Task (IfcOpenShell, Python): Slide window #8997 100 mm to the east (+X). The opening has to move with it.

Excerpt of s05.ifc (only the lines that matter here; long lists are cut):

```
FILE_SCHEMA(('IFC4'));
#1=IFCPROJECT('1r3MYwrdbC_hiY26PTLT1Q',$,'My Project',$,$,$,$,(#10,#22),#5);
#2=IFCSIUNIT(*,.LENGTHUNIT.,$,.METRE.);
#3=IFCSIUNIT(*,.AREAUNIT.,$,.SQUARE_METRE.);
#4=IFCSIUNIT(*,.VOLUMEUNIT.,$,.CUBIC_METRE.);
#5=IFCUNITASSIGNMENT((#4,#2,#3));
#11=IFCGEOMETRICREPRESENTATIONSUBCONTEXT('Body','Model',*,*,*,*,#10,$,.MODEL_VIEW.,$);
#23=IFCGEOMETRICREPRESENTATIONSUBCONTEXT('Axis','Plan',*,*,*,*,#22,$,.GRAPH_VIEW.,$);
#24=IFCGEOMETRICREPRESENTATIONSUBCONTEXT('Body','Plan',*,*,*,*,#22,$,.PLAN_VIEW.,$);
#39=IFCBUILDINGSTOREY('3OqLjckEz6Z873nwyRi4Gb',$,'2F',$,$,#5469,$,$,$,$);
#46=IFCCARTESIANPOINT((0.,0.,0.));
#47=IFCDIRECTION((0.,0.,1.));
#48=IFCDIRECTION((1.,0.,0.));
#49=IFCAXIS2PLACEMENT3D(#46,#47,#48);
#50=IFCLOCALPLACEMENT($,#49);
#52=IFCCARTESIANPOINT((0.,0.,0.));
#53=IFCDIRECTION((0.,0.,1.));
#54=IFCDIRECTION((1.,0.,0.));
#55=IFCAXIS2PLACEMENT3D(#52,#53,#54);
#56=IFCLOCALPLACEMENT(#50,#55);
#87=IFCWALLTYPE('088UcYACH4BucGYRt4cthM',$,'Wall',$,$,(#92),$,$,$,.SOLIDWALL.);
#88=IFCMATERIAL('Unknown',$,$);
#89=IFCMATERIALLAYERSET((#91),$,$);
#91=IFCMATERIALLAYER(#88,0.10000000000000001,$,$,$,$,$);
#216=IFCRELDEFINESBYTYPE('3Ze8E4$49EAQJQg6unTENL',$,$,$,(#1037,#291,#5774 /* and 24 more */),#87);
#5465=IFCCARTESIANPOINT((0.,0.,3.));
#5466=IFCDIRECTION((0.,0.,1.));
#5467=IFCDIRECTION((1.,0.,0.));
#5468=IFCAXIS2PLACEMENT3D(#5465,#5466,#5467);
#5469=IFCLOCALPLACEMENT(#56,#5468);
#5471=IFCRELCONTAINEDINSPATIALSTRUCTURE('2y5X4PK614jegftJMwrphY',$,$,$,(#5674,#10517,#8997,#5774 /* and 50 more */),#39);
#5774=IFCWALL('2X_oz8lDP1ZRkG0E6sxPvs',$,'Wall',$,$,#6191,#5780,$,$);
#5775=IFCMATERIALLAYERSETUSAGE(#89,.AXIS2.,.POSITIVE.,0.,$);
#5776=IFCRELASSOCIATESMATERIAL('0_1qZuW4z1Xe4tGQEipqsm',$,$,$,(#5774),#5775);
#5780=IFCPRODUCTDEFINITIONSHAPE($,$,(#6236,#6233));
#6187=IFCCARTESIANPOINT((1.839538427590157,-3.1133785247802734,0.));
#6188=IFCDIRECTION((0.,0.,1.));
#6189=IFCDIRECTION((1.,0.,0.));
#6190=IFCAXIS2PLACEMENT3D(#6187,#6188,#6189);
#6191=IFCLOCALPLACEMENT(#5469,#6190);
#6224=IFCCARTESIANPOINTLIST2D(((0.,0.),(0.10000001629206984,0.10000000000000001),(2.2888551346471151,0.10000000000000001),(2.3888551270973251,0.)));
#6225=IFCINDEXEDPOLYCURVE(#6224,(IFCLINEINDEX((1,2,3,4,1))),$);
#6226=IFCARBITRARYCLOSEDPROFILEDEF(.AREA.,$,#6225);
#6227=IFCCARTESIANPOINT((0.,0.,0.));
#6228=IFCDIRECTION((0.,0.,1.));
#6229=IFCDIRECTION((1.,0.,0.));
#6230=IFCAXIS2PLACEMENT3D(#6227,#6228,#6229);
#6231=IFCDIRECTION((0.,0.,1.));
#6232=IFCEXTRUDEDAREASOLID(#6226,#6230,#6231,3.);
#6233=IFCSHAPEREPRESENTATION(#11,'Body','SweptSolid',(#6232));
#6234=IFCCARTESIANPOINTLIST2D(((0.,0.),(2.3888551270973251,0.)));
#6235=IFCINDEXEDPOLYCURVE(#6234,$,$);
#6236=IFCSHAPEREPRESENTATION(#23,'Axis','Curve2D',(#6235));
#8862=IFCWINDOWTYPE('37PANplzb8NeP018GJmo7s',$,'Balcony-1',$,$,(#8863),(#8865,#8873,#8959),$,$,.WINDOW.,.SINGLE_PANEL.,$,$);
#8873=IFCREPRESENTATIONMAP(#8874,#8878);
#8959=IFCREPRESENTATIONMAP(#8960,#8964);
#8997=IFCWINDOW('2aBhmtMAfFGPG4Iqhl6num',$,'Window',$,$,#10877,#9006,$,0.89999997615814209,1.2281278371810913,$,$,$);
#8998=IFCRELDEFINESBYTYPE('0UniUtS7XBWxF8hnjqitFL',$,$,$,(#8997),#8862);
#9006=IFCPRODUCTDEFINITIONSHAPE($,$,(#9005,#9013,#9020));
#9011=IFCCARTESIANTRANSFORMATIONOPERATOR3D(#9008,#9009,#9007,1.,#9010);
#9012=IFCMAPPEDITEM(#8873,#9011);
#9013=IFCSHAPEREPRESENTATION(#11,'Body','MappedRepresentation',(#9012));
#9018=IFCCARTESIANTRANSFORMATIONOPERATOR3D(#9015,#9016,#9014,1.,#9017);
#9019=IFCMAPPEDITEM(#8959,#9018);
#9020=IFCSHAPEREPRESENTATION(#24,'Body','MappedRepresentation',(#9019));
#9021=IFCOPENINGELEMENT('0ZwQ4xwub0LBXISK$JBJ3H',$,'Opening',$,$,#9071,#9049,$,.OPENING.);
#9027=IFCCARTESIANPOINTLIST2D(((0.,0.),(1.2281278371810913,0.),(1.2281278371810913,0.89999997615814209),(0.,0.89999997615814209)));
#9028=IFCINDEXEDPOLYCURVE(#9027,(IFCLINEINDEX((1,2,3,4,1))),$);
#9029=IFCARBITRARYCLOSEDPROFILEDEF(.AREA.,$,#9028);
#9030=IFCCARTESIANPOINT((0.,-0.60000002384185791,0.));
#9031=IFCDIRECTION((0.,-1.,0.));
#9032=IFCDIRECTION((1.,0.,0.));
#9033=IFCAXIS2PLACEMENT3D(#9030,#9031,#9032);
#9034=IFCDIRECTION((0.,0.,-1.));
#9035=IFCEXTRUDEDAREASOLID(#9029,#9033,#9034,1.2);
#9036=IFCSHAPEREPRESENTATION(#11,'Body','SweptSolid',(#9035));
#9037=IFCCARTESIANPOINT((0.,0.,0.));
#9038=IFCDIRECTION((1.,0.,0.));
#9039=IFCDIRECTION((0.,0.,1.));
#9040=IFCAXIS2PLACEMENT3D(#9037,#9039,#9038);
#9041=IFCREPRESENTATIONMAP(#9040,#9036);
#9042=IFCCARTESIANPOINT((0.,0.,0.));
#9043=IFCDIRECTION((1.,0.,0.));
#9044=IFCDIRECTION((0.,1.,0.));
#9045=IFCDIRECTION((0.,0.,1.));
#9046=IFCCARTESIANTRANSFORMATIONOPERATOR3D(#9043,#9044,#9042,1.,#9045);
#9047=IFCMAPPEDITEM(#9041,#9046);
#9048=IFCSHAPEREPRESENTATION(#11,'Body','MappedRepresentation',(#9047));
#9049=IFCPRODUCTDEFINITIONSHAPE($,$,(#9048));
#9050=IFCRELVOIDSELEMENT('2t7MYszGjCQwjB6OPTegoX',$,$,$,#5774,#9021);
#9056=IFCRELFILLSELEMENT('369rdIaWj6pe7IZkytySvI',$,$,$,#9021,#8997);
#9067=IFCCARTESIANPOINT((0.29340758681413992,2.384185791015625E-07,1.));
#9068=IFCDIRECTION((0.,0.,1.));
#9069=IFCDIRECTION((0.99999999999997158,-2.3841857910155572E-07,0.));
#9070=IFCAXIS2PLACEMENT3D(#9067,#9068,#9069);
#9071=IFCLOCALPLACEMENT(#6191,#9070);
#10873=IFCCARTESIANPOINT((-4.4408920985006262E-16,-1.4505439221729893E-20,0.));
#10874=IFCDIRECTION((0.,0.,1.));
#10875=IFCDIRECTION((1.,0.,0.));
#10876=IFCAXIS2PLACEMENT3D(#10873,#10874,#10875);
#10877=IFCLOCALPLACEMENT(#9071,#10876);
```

```python
import ifcopenshell
import ifcopenshell.api.geometry
import ifcopenshell.util.placement

model = ifcopenshell.open("s05.ifc")

window = model.by_guid("2aBhmtMAfFGPG4Iqhl6num")
opening = window.FillsVoids[0].RelatingOpeningElement
wall = opening.VoidsElements[0].RelatingBuildingElement

wall_matrix = ifcopenshell.util.placement.get_local_placement(wall.ObjectPlacement)
shift = wall_matrix[:3, 0] * 0.1
before = ifcopenshell.util.placement.get_local_placement(window.ObjectPlacement)[:3, 3].copy()

# The window is placed relative to its opening, so it follows when the opening moves.
matrix = ifcopenshell.util.placement.get_local_placement(opening.ObjectPlacement)
matrix[:3, 3] += shift
ifcopenshell.api.geometry.edit_object_placement(
    model, product=opening, matrix=matrix, is_si=False, should_transform_children=True
)

after = ifcopenshell.util.placement.get_local_placement(window.ObjectPlacement)[:3, 3]
print("window moved by", (after - before).round(3) + 0.0)

model.write("s05_rev.ifc")
```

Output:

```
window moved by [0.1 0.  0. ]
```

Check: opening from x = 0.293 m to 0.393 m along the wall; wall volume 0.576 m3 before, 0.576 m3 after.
